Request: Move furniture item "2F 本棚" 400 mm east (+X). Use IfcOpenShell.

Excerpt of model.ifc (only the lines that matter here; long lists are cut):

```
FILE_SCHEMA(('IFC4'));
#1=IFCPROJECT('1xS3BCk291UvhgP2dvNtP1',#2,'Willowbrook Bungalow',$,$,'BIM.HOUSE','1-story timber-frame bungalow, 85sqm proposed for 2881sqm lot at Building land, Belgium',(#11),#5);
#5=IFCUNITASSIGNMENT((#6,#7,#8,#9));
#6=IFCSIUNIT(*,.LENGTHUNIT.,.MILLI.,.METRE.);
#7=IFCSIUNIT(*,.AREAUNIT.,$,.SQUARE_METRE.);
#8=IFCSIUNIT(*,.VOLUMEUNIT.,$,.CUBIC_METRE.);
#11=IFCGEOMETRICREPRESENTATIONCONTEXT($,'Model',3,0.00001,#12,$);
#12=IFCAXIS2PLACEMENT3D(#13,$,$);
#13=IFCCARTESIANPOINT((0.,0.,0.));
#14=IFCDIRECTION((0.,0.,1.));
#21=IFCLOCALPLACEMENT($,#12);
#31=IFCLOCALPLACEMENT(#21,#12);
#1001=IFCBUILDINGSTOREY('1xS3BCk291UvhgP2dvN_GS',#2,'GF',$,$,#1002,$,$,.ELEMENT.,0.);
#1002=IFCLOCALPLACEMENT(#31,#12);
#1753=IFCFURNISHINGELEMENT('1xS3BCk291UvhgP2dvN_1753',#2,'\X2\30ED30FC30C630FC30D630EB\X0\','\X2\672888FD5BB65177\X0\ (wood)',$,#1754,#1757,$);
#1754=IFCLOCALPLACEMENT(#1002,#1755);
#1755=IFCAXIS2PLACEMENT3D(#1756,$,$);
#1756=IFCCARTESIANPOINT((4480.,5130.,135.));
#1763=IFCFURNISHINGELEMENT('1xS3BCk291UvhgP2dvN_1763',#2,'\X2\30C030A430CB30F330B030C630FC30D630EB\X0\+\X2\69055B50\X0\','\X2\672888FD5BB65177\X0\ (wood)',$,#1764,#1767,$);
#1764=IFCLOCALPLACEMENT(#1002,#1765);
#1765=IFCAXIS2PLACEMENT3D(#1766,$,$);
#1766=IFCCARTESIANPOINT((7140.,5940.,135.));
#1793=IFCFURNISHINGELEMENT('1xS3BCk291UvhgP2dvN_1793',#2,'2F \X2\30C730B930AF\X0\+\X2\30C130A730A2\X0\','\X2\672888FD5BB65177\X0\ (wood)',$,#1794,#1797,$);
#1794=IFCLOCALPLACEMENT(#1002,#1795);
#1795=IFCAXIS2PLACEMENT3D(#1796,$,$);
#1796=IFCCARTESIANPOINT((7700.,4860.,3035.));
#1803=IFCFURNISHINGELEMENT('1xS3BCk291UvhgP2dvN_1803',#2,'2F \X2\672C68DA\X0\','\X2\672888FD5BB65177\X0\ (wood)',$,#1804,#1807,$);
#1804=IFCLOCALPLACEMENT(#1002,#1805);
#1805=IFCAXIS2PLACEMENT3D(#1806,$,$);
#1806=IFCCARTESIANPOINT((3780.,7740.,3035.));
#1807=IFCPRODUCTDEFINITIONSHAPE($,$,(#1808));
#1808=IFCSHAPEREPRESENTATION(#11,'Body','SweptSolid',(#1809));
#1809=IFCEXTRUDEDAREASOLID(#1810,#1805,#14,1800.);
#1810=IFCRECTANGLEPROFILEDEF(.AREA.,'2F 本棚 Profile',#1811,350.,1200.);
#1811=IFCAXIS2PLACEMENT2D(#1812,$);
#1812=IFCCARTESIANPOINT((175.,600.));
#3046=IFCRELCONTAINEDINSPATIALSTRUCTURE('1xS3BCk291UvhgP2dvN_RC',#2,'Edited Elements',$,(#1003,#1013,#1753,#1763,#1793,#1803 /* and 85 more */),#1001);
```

```python
import ifcopenshell
import ifcopenshell.api.geometry
import ifcopenshell.util.placement
import ifcopenshell.util.unit

model = ifcopenshell.open("model.ifc")
unit_scale = ifcopenshell.util.unit.calculate_unit_scale(model)

item = model.by_guid("1xS3BCk291UvhgP2dvN_1803")
matrix = ifcopenshell.util.placement.get_local_placement(item.ObjectPlacement)
matrix[0, 3] += 0.4 / unit_scale
ifcopenshell.api.geometry.edit_object_placement(model, product=item, matrix=matrix, is_si=False)

print(ifcopenshell.util.placement.get_local_placement(item.ObjectPlacement).round(3) + 0.0)

model.write("model_v2.ifc")
```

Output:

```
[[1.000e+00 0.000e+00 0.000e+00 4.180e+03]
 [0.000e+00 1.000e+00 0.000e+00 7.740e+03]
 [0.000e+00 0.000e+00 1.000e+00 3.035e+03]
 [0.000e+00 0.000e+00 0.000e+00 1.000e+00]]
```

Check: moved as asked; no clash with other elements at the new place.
